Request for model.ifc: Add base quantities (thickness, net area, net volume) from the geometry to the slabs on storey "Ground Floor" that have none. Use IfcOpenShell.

First a look at what the model holds.

```python
import ifcopenshell
import ifcopenshell.util.element
import ifcopenshell.util.unit

model = ifcopenshell.open("model.ifc")
print(model.schema)
for unit_type in ("LENGTHUNIT", "AREAUNIT", "VOLUMEUNIT"):
    print(unit_type, ifcopenshell.util.unit.calculate_unit_scale(model, unit_type))
storey = next(s for s in model.by_type("IfcBuildingStorey") if s.Name == "Ground Floor")
slabs = [e for e in ifcopenshell.util.element.get_decomposition(storey) if e.is_a("IfcSlab")]
for e in sorted(slabs, key=lambda e: e.id()):
    print(e.id(), e.is_a(), e.Name, list(ifcopenshell.util.element.get_psets(e, qtos_only=True)), sep=" | ")
```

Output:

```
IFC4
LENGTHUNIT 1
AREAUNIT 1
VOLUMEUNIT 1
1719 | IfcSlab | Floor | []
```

```python
import ifcopenshell
import ifcopenshell.api.pset
import ifcopenshell.geom
import ifcopenshell.util.element
import ifcopenshell.util.shape
import ifcopenshell.util.unit

model = ifcopenshell.open("model.ifc")
unit_scale = ifcopenshell.util.unit.calculate_unit_scale(model)
area_scale = ifcopenshell.util.unit.calculate_unit_scale(model, "AREAUNIT")
volume_scale = ifcopenshell.util.unit.calculate_unit_scale(model, "VOLUMEUNIT")
settings = ifcopenshell.geom.settings()

storey = next(s for s in model.by_type("IfcBuildingStorey") if s.Name == "Ground Floor")
slabs = [e for e in ifcopenshell.util.element.get_decomposition(storey) if e.is_a("IfcSlab")]

for e in sorted(slabs, key=lambda e: e.id()):
    if ifcopenshell.util.element.get_psets(e, qtos_only=True, should_inherit=False):
        continue
    # Geometry comes back in metres, in the element's own axes.
    shape = ifcopenshell.geom.create_shape(settings, e)
    values = {
        "Width": ifcopenshell.util.shape.get_z(shape.geometry) / unit_scale,
        "NetArea": ifcopenshell.util.shape.get_footprint_area(shape.geometry) / area_scale,
        "NetVolume": ifcopenshell.util.shape.get_volume(shape.geometry) / volume_scale,
    }
    qto = ifcopenshell.api.pset.add_qto(model, product=e, name="Qto_SlabBaseQuantities")
    ifcopenshell.api.pset.edit_qto(model, qto=qto, properties=values)
    print(e.id(), {k: round(v, 3) for k, v in values.items()})

model.write("model_v2.ifc")
```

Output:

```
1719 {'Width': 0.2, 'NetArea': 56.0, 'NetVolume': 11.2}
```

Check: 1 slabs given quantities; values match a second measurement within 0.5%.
